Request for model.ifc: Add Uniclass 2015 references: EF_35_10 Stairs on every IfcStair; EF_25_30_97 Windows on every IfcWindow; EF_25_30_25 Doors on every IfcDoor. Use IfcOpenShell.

First a look at what the model holds.

```python
import ifcopenshell

model = ifcopenshell.open("model.ifc")
print(model.schema)
print("classifications:", [c.Name for c in model.by_type("IfcClassification")])
for ifc_class in ("IfcDoor", "IfcRoof", "IfcStair", "IfcWall", "IfcWindow"):
    print(ifc_class, len(model.by_type(ifc_class)))
```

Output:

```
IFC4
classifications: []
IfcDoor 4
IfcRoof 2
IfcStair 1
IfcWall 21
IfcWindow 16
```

```python
import ifcopenshell
import ifcopenshell.api.classification

model = ifcopenshell.open("model.ifc")

system = ifcopenshell.api.classification.add_classification(model, classification="Uniclass 2015")

codes = {
    "IfcStair": ("EF_35_10", "Stairs"),
    "IfcWindow": ("EF_25_30_97", "Windows"),
    "IfcDoor": ("EF_25_30_25", "Doors"),
}
for ifc_class, (code, name) in codes.items():
    products = model.by_type(ifc_class)
    ifcopenshell.api.classification.add_reference(
        model, products=products, classification=system, identification=code, name=name
    )
    print(code, len(products))

model.write("model_updated.ifc")
```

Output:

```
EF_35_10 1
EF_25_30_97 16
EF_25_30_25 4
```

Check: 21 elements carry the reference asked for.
